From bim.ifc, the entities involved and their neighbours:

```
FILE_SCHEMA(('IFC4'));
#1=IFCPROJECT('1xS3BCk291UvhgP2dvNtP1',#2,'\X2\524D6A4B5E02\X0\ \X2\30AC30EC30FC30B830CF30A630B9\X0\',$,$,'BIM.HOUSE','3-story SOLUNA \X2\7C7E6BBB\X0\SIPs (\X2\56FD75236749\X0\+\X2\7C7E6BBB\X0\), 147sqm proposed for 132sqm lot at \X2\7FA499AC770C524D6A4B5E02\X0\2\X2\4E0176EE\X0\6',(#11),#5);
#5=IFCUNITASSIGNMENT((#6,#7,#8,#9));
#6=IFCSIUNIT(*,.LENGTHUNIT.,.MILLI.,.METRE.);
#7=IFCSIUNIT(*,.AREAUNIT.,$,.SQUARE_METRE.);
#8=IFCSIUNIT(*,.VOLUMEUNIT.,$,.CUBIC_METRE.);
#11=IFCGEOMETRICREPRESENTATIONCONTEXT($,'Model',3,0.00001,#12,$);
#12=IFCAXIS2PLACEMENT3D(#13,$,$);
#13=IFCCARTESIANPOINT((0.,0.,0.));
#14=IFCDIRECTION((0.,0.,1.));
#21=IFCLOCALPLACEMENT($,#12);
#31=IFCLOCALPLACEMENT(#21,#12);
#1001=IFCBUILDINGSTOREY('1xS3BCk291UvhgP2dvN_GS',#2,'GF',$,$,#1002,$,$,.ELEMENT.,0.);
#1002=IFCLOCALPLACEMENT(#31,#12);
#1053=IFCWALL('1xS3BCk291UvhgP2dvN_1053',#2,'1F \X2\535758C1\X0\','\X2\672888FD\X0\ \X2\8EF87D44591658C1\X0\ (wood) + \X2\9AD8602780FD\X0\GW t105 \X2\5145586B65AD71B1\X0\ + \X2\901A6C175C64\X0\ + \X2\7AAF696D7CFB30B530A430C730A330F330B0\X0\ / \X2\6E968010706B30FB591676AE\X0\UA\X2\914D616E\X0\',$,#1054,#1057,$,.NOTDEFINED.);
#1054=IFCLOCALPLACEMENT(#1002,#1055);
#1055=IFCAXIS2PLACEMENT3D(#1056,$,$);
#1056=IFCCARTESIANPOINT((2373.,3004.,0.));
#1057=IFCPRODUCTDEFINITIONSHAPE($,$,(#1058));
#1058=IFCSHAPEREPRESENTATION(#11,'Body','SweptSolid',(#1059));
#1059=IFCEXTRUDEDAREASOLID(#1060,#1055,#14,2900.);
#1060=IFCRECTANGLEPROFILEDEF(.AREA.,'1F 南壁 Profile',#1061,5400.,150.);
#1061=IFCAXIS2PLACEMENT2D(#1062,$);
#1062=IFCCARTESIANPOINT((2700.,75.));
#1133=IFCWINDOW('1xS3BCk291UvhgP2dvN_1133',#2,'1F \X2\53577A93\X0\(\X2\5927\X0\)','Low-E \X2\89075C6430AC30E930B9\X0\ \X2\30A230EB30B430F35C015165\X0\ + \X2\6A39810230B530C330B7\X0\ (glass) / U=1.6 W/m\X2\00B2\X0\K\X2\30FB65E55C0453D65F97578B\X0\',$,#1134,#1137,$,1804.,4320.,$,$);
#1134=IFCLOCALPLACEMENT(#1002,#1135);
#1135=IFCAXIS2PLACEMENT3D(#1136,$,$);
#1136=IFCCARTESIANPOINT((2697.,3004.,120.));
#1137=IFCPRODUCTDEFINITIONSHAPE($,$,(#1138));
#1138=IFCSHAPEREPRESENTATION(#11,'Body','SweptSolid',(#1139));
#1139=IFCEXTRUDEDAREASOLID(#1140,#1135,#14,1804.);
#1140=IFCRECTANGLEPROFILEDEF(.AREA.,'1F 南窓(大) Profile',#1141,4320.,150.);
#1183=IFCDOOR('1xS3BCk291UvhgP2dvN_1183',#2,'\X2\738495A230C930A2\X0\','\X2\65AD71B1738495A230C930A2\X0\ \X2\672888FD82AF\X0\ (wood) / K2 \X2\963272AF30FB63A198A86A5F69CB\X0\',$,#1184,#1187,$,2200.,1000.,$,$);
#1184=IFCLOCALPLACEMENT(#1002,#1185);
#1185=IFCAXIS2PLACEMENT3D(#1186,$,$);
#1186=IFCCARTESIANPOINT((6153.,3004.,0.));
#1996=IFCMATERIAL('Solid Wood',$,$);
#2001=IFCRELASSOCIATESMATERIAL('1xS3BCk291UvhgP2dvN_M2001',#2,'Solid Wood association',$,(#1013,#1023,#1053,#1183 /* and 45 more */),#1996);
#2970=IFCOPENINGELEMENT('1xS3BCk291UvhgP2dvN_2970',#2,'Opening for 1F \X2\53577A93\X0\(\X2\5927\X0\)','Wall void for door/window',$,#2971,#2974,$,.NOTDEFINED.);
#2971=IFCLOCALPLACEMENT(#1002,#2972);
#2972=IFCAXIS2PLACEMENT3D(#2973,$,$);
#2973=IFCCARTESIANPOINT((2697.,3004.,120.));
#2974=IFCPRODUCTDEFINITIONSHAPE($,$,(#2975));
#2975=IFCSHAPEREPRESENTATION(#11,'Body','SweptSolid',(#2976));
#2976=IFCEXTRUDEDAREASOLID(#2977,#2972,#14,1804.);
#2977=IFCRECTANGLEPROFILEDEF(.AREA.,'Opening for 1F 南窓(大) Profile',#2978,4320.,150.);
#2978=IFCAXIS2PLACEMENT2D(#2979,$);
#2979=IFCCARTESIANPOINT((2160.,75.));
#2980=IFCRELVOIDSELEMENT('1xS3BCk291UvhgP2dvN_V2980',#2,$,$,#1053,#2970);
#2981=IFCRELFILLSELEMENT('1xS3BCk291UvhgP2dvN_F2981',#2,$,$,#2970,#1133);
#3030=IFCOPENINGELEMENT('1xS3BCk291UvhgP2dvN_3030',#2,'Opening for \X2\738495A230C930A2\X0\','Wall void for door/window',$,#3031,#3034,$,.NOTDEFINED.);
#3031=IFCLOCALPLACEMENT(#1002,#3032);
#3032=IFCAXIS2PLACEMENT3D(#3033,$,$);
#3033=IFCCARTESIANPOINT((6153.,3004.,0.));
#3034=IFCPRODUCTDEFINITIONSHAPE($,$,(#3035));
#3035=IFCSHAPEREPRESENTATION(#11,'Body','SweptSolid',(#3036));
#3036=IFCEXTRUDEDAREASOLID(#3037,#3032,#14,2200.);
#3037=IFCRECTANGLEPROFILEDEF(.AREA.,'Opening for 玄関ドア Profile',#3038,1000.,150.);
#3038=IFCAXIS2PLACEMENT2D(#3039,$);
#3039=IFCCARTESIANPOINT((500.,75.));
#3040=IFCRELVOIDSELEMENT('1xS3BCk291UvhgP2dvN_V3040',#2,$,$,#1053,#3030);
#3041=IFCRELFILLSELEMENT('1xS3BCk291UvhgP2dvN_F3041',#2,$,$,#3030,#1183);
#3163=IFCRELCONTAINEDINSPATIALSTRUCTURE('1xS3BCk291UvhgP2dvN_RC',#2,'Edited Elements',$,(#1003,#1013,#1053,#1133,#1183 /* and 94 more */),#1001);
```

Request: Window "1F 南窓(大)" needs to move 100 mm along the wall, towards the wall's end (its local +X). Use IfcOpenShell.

```python
import ifcopenshell
import ifcopenshell.api.geometry
import ifcopenshell.util.placement
import ifcopenshell.util.unit

model = ifcopenshell.open("bim.ifc")
unit_scale = ifcopenshell.util.unit.calculate_unit_scale(model)

window = model.by_guid("1xS3BCk291UvhgP2dvN_1133")
opening = window.FillsVoids[0].RelatingOpeningElement
wall = opening.VoidsElements[0].RelatingBuildingElement

wall_matrix = ifcopenshell.util.placement.get_local_placement(wall.ObjectPlacement)
shift = wall_matrix[:3, 0] * 0.1 / unit_scale
before = ifcopenshell.util.placement.get_local_placement(window.ObjectPlacement)[:3, 3].copy()

# The window is not placed relative to its opening, so move both.
for product in (opening, window):
    matrix = ifcopenshell.util.placement.get_local_placement(product.ObjectPlacement)
    matrix[:3, 3] += shift
    ifcopenshell.api.geometry.edit_object_placement(model, product=product, matrix=matrix, is_si=False)

after = ifcopenshell.util.placement.get_local_placement(window.ObjectPlacement)[:3, 3]
print("window moved by", (after - before).round(3) + 0.0)

model.write("bim_rev.ifc")
```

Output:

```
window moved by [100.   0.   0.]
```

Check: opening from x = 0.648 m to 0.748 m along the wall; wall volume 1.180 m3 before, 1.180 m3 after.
